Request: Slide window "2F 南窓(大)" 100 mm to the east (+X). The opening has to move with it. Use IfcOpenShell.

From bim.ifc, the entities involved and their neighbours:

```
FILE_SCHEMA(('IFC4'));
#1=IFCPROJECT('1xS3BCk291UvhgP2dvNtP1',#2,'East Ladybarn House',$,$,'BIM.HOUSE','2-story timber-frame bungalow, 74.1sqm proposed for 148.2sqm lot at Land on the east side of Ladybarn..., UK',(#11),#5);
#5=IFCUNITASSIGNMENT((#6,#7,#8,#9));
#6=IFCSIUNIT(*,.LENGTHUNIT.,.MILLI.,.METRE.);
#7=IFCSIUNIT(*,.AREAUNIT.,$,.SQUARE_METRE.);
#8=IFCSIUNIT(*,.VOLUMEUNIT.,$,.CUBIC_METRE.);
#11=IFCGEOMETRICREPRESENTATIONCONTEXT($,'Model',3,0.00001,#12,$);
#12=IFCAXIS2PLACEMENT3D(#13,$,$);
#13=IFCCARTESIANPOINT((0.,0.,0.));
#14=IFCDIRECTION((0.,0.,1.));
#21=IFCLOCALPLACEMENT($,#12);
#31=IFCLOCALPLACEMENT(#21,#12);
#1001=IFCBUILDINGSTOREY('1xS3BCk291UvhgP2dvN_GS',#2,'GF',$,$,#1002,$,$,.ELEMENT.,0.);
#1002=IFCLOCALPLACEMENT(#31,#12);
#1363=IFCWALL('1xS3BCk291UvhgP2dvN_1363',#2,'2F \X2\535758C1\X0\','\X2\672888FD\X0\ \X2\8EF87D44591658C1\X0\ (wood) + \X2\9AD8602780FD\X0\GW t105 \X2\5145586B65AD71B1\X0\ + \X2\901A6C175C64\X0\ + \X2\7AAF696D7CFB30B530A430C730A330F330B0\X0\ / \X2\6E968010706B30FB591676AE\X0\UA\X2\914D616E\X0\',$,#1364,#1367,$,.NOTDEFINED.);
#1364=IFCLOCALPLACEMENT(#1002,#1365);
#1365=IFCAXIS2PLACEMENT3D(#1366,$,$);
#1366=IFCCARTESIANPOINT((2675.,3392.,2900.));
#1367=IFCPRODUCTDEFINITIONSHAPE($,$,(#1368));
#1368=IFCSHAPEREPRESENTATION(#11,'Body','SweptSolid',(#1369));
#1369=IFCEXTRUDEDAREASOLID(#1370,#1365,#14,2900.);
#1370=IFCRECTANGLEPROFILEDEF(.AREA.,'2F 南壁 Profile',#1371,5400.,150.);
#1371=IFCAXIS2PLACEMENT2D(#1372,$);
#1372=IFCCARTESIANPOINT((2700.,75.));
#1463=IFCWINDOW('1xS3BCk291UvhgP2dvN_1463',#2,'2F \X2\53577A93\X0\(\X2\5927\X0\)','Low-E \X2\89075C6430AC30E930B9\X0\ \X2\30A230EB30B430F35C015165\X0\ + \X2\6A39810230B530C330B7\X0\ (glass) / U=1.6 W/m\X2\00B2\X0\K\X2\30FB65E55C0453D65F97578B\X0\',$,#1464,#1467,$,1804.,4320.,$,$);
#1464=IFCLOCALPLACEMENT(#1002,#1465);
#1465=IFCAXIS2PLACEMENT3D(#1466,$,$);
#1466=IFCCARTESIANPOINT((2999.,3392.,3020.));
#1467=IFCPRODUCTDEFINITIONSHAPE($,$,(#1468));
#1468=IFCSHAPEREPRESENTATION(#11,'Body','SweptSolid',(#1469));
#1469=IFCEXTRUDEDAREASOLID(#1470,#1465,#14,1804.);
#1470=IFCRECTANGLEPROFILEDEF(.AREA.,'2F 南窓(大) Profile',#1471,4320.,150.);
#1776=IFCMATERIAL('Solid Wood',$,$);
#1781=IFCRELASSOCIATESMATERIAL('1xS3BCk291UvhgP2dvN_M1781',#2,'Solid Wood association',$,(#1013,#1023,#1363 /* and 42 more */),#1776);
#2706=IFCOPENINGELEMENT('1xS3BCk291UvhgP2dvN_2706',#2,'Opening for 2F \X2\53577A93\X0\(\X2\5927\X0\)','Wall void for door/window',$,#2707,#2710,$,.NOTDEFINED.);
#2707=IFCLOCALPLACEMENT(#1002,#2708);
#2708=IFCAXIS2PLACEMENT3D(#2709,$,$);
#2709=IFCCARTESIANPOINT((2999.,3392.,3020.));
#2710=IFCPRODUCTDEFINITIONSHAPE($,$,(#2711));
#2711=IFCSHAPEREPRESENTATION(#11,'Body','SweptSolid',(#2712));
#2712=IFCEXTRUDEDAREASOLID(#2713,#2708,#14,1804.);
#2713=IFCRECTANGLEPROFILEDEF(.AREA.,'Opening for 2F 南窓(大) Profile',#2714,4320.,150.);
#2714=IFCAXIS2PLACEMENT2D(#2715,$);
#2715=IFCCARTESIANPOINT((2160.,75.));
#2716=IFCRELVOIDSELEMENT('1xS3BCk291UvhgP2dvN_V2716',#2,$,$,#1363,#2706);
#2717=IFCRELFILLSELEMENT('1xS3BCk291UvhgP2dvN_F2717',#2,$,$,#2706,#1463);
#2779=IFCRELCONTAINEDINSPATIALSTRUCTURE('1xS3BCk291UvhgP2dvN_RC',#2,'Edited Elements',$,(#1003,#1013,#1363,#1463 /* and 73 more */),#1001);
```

```python
import ifcopenshell
import ifcopenshell.api.geometry
import ifcopenshell.util.placement

model = ifcopenshell.open("bim.ifc")

window = model.by_guid("1xS3BCk291UvhgP2dvN_1463")
opening = window.FillsVoids[0].RelatingOpeningElement
wall = opening.VoidsElements[0].RelatingBuildingElement

wall_matrix = ifcopenshell.util.placement.get_local_placement(wall.ObjectPlacement)
shift = wall_matrix[:3, 0] * 100.0
before = ifcopenshell.util.placement.get_local_placement(window.ObjectPlacement)[:3, 3].copy()

# The window is not placed relative to its opening, so move both.
for product in (opening, window):
    matrix = ifcopenshell.util.placement.get_local_placement(product.ObjectPlacement)
    matrix[:3, 3] += shift
    ifcopenshell.api.geometry.edit_object_placement(model, product=product, matrix=matrix, is_si=False)

after = ifcopenshell.util.placement.get_local_placement(window.ObjectPlacement)[:3, 3]
print("window moved by", (after - before).round(3) + 0.0)

model.write("bim_updated.ifc")
```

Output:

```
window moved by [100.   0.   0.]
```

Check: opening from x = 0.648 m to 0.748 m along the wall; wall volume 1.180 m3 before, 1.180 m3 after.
